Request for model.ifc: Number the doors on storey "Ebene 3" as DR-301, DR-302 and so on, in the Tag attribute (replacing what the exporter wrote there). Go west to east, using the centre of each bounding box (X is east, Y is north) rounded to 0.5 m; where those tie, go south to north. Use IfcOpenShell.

First a look at what the model holds.

```python
import ifcopenshell
import ifcopenshell.util.element
import ifcopenshell.util.placement

model = ifcopenshell.open("model.ifc")
print(model.schema)
storey = next(s for s in model.by_type("IfcBuildingStorey") if s.Name == "Ebene 3")
doors = [e for e in ifcopenshell.util.element.get_decomposition(storey) if e.is_a("IfcDoor")]
for e in sorted(doors, key=lambda e: e.id()):
    origin = ifcopenshell.util.placement.get_local_placement(e.ObjectPlacement)[:3, 3]
    print(e.id(), e.Tag, e.Name, origin.round(2) + 0.0, sep=" | ")
```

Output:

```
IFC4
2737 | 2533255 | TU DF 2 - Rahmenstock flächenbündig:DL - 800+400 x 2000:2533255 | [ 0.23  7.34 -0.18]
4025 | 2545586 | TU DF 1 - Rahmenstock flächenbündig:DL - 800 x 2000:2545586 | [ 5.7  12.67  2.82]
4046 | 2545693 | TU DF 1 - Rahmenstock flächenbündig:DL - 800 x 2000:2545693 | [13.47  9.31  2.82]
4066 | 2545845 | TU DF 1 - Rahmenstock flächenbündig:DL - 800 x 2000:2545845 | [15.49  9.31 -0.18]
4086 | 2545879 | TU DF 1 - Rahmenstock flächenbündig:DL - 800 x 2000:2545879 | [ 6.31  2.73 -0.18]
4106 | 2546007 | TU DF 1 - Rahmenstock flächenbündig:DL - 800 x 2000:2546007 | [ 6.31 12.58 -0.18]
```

```python
import ifcopenshell
import ifcopenshell.geom
import ifcopenshell.util.element
import ifcopenshell.util.shape

model = ifcopenshell.open("model.ifc")
settings = ifcopenshell.geom.settings()
settings.set("use-world-coords", True)


def centre(element):
    shape = ifcopenshell.geom.create_shape(settings, element)
    return ifcopenshell.util.shape.get_bbox_centroid(shape.geometry)


storey = next(s for s in model.by_type("IfcBuildingStorey") if s.Name == "Ebene 3")
doors = [e for e in ifcopenshell.util.element.get_decomposition(storey) if e.is_a("IfcDoor")]

# Insertion points can sit at a corner or the storey origin, so sort by the geometry (in metres).
centres = {e: centre(e) for e in doors}
doors.sort(key=lambda e: (round(centres[e][0] / 0.5), centres[e][1]))

for i, e in enumerate(doors, start=1):
    number = f"DR-3{i:02d}"
    e.Tag = number
    print(e.id(), number)

model.write("model_updated.ifc")
```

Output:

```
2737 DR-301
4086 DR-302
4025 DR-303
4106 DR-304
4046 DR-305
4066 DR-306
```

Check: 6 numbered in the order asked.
